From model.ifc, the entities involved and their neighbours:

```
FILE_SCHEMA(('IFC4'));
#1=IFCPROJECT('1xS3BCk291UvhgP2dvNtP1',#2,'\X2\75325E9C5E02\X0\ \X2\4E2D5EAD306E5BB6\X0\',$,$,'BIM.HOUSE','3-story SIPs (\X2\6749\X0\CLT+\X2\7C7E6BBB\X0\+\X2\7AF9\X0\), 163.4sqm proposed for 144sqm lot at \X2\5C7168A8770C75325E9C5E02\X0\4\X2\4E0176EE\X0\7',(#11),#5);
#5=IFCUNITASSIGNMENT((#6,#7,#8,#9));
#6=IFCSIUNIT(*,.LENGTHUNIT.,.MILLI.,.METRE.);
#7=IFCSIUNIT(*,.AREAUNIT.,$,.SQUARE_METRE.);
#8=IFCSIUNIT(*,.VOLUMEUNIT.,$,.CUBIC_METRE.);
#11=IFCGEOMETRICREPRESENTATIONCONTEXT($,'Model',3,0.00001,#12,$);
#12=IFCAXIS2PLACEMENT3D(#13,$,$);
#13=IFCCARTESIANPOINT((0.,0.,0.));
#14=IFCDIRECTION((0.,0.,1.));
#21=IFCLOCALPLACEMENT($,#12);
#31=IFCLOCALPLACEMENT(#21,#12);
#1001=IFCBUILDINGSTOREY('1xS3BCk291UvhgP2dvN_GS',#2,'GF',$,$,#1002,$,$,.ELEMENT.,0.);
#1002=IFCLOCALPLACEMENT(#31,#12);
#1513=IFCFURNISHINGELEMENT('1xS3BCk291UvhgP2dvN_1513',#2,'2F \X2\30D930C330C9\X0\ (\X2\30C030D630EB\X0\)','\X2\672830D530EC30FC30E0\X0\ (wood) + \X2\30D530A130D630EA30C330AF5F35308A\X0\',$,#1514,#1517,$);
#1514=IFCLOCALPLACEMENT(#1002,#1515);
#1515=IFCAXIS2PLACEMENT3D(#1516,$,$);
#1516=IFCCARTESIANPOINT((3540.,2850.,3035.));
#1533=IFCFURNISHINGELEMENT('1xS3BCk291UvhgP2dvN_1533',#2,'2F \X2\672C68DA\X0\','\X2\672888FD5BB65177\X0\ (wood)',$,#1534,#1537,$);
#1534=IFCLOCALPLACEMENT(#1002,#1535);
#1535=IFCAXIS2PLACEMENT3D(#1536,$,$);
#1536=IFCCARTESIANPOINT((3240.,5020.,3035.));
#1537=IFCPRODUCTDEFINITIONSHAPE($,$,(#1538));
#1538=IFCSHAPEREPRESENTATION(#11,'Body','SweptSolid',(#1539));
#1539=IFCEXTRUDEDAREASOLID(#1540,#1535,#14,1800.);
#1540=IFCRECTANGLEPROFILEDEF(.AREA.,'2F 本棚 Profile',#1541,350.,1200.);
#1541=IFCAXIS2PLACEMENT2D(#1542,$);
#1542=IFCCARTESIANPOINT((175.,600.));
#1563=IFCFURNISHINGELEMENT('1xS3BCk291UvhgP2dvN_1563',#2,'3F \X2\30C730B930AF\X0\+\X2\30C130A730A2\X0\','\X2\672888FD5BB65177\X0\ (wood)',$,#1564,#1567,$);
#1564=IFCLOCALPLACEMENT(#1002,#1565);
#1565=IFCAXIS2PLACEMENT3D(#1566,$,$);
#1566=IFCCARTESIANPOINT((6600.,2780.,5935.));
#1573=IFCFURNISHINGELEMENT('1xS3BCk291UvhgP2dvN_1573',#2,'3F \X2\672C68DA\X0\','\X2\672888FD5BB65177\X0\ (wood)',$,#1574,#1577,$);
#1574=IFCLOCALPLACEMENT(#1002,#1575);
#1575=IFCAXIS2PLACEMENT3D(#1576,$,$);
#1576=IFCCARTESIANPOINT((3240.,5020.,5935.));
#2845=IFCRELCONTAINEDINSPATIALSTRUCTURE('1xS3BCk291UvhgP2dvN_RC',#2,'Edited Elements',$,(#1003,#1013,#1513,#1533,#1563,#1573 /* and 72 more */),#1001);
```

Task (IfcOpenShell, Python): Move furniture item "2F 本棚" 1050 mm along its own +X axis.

```python
import ifcopenshell
import ifcopenshell.api.geometry
import ifcopenshell.util.placement

model = ifcopenshell.open("model.ifc")

item = model.by_guid("1xS3BCk291UvhgP2dvN_1533")
matrix = ifcopenshell.util.placement.get_local_placement(item.ObjectPlacement)
matrix[:3, 3] += matrix[:3, 0] * 1050.0
ifcopenshell.api.geometry.edit_object_placement(model, product=item, matrix=matrix, is_si=False)

print(ifcopenshell.util.placement.get_local_placement(item.ObjectPlacement).round(3) + 0.0)

model.write("model_v2.ifc")
```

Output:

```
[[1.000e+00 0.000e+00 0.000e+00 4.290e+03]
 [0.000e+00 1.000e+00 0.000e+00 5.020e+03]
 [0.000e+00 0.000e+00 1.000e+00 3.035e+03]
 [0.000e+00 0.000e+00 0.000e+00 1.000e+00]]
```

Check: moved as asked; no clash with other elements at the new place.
